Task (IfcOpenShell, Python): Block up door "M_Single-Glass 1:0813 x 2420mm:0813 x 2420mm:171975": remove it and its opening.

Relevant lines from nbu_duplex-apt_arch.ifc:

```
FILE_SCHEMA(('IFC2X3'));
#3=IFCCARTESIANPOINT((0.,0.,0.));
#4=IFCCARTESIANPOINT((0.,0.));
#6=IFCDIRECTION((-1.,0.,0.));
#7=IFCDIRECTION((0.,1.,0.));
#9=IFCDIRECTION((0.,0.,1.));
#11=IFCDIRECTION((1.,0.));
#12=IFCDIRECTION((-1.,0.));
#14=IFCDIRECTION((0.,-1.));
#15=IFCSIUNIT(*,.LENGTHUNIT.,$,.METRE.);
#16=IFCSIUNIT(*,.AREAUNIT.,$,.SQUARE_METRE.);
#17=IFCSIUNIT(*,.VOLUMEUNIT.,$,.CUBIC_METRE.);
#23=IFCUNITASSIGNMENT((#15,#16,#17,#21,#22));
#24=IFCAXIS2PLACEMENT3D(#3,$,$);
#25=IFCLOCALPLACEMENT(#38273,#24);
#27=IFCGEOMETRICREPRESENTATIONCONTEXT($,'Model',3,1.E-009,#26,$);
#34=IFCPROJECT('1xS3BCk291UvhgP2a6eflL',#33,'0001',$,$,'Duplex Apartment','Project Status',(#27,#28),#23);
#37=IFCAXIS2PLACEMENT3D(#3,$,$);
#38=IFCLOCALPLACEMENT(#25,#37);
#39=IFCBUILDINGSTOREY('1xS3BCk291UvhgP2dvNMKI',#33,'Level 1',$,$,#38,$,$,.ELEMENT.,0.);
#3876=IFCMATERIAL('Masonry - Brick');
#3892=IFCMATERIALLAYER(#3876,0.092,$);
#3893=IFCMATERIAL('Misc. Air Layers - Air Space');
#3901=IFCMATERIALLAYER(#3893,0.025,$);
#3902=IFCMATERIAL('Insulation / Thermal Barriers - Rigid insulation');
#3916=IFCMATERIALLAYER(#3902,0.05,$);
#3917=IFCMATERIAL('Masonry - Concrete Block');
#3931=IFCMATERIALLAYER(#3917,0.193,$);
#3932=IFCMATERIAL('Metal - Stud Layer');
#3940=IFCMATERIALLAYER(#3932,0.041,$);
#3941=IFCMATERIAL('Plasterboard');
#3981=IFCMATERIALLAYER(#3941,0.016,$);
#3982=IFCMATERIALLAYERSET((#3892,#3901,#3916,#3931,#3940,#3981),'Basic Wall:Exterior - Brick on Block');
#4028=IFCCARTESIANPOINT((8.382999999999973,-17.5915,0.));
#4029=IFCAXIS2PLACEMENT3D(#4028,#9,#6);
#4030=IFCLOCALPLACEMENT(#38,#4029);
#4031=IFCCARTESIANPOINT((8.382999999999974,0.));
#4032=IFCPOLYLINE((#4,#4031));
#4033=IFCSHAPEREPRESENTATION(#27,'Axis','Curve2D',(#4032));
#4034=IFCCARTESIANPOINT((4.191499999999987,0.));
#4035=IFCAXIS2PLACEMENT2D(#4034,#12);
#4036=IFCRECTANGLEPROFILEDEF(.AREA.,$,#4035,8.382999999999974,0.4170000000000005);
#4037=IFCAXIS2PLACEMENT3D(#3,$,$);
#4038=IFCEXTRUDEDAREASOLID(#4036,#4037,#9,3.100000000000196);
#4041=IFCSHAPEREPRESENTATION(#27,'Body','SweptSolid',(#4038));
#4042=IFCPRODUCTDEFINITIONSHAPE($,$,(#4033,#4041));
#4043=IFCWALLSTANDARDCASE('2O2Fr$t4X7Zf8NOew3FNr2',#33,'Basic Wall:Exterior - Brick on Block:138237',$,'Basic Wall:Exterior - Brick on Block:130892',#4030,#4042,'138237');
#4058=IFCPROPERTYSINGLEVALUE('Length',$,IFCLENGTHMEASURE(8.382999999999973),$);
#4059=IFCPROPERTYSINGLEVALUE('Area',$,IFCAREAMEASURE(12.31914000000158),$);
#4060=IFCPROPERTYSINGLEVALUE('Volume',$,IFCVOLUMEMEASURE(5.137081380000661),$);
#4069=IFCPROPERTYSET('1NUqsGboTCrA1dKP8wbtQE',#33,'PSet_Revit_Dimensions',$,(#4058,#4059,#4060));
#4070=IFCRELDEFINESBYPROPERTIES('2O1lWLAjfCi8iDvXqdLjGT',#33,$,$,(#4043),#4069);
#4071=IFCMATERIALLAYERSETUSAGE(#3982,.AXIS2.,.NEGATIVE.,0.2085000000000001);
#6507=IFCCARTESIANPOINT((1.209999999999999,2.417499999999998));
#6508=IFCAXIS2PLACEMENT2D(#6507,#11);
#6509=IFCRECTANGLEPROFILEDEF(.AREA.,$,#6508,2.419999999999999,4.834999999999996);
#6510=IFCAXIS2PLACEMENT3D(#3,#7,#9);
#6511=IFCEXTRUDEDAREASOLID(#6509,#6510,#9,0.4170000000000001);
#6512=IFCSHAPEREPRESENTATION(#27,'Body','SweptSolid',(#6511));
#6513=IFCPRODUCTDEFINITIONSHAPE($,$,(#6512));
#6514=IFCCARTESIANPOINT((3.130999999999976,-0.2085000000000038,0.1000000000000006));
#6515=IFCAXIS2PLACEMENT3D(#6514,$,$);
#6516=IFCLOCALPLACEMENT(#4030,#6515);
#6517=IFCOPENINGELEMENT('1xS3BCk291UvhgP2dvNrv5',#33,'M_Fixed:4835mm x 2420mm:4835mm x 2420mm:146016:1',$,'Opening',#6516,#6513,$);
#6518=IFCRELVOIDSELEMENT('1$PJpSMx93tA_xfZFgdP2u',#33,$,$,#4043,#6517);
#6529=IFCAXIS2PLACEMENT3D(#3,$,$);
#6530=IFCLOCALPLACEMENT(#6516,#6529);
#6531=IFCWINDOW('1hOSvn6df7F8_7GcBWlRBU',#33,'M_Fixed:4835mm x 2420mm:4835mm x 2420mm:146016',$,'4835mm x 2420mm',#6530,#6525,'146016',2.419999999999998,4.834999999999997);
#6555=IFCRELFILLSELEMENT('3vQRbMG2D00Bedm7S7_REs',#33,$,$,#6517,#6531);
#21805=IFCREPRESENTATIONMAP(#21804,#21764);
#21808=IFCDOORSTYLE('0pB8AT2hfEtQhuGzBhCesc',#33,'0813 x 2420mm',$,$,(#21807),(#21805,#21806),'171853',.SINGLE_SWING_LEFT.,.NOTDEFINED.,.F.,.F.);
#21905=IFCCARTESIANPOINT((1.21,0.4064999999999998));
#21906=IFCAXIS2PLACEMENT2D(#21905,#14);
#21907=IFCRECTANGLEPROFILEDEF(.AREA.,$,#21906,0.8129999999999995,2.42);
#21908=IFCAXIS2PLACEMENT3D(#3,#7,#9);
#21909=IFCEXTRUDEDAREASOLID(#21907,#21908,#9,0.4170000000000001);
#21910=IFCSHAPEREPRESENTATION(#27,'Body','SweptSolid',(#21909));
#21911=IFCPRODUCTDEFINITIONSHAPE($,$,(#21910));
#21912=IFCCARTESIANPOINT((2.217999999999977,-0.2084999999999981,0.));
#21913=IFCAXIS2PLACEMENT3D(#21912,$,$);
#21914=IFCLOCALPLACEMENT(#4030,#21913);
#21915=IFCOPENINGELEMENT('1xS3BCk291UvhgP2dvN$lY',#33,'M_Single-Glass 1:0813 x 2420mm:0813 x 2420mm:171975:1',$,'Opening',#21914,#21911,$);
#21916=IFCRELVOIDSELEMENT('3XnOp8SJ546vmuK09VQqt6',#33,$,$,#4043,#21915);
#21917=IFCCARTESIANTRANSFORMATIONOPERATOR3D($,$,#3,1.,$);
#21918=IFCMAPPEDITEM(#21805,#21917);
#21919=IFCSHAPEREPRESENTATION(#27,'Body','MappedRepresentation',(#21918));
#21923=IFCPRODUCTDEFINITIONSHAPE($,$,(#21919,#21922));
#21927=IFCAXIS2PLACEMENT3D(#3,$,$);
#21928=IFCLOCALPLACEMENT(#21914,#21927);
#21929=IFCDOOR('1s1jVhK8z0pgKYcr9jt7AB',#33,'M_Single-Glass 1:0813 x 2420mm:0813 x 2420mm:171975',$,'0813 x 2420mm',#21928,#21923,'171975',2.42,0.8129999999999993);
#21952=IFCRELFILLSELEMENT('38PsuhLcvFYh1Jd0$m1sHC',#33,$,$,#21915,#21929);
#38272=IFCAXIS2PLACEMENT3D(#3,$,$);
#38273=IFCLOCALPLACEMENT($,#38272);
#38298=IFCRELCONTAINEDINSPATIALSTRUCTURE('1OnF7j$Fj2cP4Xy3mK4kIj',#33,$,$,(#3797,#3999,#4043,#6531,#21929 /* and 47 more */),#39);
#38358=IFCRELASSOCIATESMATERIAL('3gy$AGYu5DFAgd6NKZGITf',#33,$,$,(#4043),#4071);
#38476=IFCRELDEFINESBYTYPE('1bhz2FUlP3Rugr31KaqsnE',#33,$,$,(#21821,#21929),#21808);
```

```python
import ifcopenshell
import ifcopenshell.api.feature
import ifcopenshell.api.pset
import ifcopenshell.api.root
import ifcopenshell.geom
import ifcopenshell.util.element
import ifcopenshell.util.shape
import ifcopenshell.util.unit

model = ifcopenshell.open("nbu_duplex-apt_arch.ifc")
area_scale = ifcopenshell.util.unit.calculate_unit_scale(model, "AREAUNIT")
volume_scale = ifcopenshell.util.unit.calculate_unit_scale(model, "VOLUMEUNIT")
settings = ifcopenshell.geom.settings()


def volume(element):
    """Net volume in cubic metres, openings subtracted."""
    shape = ifcopenshell.geom.create_shape(settings, element)
    return ifcopenshell.util.shape.get_volume(shape.geometry)


door = model.by_guid("1s1jVhK8z0pgKYcr9jt7AB")
opening = door.FillsVoids[0].RelatingOpeningElement
wall = opening.VoidsElements[0].RelatingBuildingElement
before = volume(wall)

ifcopenshell.api.root.remove_product(model, product=door)
ifcopenshell.api.feature.remove_feature(model, feature=opening)

after = volume(wall)
thickness = 0.417  # wall thickness in metres

# Update the wall's stored quantities.
pset = model.by_id(ifcopenshell.util.element.get_pset(wall, "PSet_Revit_Dimensions", should_inherit=False)["id"])
ifcopenshell.api.pset.edit_pset(model, pset=pset, properties={
    "Area": model.create_entity("IfcAreaMeasure", after / thickness / area_scale),
    "Volume": model.create_entity("IfcVolumeMeasure", after / volume_scale),
})

print(f"wall volume {before:.3f} -> {after:.3f} m3")

model.write("nbu_duplex-apt_arch-out.ifc")
```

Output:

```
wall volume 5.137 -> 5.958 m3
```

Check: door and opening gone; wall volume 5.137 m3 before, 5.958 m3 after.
